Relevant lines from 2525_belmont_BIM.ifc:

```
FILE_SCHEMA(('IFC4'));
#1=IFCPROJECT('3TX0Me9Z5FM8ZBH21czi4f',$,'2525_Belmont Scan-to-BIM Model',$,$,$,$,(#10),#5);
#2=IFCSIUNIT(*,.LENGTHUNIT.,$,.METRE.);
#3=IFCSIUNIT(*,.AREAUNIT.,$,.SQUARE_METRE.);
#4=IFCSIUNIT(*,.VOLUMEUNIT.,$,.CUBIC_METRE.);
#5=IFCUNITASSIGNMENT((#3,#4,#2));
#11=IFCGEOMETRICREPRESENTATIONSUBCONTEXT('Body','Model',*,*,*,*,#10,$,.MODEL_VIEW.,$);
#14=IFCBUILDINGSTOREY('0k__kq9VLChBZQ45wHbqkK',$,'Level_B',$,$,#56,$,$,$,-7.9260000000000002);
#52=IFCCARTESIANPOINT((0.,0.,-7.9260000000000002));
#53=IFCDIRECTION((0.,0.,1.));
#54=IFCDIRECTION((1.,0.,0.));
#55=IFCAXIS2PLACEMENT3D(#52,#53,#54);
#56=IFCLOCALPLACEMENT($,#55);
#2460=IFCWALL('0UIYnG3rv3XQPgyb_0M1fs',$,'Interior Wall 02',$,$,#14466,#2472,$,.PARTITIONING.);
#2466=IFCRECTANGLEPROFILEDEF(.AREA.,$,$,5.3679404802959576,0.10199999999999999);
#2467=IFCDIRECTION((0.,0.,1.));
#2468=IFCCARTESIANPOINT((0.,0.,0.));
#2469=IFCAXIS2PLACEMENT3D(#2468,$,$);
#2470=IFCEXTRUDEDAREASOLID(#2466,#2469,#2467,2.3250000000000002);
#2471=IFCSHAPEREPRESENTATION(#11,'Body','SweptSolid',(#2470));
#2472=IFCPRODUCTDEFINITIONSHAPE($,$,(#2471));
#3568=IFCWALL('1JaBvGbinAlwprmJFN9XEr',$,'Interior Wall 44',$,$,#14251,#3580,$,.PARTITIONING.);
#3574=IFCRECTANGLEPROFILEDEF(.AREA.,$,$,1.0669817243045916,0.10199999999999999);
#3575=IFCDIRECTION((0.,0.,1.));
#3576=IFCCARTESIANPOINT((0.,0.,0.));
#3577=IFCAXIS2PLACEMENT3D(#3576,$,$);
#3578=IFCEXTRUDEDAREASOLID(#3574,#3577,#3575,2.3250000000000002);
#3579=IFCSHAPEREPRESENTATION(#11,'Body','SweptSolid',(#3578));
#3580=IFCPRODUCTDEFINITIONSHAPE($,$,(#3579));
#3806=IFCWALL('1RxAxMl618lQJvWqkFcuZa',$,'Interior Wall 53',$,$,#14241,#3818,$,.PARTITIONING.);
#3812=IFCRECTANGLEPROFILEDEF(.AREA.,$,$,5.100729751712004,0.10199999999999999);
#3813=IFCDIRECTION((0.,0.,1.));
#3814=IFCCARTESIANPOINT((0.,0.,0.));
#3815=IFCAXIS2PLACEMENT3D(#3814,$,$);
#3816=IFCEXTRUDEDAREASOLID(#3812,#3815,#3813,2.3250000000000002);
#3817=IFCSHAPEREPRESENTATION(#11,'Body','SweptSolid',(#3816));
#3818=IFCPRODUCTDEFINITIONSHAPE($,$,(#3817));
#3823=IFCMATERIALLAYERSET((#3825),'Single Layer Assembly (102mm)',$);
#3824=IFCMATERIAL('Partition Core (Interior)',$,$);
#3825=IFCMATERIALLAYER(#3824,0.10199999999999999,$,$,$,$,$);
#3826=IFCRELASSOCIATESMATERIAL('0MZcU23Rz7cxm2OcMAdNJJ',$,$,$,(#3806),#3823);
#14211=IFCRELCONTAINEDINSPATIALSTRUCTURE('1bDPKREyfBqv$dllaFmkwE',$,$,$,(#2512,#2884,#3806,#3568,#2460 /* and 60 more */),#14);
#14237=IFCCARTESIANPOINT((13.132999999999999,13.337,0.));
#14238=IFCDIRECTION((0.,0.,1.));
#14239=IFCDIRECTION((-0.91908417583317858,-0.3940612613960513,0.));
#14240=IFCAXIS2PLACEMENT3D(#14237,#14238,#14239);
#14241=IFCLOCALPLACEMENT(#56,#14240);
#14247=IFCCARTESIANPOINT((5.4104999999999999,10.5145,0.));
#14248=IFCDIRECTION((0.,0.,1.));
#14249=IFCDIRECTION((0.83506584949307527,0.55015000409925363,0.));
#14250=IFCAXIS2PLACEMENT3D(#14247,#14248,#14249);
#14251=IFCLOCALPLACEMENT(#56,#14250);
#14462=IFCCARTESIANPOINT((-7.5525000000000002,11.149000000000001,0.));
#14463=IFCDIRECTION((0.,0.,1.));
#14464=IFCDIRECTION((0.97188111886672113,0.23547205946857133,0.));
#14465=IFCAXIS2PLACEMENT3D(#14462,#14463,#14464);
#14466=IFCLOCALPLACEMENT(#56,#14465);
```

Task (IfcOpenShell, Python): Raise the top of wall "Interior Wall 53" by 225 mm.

```python
import ifcopenshell
import ifcopenshell.geom
import ifcopenshell.util.representation
import ifcopenshell.util.shape
import ifcopenshell.util.unit

model = ifcopenshell.open("2525_belmont_BIM.ifc")
unit_scale = ifcopenshell.util.unit.calculate_unit_scale(model)
settings = ifcopenshell.geom.settings()


def volume(element):
    """Net volume in cubic metres, openings subtracted."""
    shape = ifcopenshell.geom.create_shape(settings, element)
    return ifcopenshell.util.shape.get_volume(shape.geometry)


wall = model.by_id(3806)
before = volume(wall)

body = ifcopenshell.util.representation.get_representation(wall, "Model", "Body")
solid = body.Items[0]
old_height = solid.Depth
solid.Depth += 0.225 / unit_scale
after = volume(wall)

print(f"height {old_height:g} -> {solid.Depth:g}, volume {before:.3f} -> {after:.3f} m3")

model.write("2525_belmont_BIM_rev.ifc")
```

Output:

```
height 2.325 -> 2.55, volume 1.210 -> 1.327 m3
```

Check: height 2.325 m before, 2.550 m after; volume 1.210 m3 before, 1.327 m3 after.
